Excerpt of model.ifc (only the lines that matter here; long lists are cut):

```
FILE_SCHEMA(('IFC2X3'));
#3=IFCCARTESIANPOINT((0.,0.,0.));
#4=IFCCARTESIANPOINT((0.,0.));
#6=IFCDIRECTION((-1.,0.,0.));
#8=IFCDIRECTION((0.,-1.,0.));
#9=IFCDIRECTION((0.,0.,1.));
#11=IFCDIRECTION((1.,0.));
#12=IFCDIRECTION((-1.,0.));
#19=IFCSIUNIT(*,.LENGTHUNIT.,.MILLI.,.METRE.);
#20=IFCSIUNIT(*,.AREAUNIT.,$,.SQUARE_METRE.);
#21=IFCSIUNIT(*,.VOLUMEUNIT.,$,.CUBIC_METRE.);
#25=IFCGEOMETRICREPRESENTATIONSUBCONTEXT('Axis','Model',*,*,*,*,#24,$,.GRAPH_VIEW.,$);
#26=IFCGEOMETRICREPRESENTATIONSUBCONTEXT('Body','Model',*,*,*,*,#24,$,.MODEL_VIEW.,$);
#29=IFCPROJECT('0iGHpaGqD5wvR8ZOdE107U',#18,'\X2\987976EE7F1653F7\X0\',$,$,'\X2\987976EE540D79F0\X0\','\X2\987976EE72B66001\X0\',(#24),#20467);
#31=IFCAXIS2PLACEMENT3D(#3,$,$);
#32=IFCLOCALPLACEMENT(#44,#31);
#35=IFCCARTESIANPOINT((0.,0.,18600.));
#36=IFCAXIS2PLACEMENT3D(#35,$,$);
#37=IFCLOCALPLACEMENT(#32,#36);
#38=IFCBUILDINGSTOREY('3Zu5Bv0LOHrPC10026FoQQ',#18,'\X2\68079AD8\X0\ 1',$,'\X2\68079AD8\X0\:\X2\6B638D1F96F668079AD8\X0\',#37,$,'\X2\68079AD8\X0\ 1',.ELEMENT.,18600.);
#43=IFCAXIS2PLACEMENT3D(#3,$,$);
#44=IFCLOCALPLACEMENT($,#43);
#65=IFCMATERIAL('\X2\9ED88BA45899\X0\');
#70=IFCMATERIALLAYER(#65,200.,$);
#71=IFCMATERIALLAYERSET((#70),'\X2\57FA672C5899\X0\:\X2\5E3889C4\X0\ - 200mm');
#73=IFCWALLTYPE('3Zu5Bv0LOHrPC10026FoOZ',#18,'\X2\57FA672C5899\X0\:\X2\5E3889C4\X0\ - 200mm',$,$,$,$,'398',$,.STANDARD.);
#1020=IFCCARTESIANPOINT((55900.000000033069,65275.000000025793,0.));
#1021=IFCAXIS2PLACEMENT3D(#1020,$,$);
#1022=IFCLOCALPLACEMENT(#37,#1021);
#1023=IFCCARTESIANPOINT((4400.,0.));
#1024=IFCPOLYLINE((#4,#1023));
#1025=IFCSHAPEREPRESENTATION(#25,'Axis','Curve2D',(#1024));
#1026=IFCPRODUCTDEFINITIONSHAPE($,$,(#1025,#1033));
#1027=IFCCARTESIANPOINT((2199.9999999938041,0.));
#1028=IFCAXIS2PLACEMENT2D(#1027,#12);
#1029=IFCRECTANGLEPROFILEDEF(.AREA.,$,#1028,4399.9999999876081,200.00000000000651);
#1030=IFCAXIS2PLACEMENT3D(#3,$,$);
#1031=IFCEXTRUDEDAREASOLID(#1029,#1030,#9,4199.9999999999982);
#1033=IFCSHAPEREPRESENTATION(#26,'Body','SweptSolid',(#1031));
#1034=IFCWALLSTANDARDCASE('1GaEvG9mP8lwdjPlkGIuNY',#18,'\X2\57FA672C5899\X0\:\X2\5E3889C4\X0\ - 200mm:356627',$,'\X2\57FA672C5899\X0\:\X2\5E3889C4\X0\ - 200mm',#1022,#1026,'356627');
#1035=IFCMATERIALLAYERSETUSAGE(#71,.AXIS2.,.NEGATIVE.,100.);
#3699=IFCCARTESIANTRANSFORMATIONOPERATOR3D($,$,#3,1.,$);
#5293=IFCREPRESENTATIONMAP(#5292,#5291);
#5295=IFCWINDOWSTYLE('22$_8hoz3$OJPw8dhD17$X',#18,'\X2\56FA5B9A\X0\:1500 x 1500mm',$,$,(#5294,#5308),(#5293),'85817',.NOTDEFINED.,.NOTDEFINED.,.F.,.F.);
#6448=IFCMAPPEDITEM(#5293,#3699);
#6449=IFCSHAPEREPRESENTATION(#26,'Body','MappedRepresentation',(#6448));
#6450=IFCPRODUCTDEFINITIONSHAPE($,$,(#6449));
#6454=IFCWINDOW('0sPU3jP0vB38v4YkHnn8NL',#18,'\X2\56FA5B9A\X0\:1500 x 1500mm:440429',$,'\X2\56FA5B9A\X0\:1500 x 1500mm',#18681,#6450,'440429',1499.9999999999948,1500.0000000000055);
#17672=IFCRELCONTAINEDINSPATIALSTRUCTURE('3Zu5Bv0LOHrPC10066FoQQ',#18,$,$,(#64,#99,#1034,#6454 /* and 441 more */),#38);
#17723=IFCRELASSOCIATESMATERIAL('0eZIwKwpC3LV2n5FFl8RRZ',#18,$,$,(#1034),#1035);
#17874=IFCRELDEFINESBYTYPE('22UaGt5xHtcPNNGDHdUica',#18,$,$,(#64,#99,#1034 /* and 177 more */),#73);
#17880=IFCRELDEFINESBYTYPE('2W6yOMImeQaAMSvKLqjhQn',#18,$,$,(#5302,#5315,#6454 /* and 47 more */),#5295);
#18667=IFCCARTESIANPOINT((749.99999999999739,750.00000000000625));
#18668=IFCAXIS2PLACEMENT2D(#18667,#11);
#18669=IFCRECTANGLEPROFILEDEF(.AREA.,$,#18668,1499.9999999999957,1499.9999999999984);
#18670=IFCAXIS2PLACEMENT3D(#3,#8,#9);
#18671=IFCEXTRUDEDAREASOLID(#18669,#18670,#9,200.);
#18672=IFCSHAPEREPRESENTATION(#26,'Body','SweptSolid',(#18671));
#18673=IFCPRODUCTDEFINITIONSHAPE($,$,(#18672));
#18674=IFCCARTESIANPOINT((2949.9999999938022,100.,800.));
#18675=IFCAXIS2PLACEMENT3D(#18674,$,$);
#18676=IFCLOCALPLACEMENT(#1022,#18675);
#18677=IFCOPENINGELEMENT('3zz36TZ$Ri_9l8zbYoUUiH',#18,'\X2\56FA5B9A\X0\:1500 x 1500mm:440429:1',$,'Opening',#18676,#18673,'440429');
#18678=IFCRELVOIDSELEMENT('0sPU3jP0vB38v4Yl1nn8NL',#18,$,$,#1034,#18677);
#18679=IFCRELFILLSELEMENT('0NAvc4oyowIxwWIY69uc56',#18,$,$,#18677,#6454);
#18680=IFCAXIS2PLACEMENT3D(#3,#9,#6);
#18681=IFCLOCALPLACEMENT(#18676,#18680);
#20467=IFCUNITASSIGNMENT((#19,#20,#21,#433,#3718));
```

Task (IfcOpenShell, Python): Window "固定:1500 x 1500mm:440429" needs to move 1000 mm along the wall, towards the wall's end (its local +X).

```python
import ifcopenshell
import ifcopenshell.api.geometry
import ifcopenshell.util.placement
import ifcopenshell.util.unit

model = ifcopenshell.open("model.ifc")
unit_scale = ifcopenshell.util.unit.calculate_unit_scale(model)

window = model.by_id(6454)
opening = window.FillsVoids[0].RelatingOpeningElement
wall = opening.VoidsElements[0].RelatingBuildingElement

wall_matrix = ifcopenshell.util.placement.get_local_placement(wall.ObjectPlacement)
shift = wall_matrix[:3, 0] * 1 / unit_scale
before = ifcopenshell.util.placement.get_local_placement(window.ObjectPlacement)[:3, 3].copy()

# The window is placed relative to its opening, so it follows when the opening moves.
matrix = ifcopenshell.util.placement.get_local_placement(opening.ObjectPlacement)
matrix[:3, 3] += shift
ifcopenshell.api.geometry.edit_object_placement(
    model, product=opening, matrix=matrix, is_si=False, should_transform_children=True
)

after = ifcopenshell.util.placement.get_local_placement(window.ObjectPlacement)[:3, 3]
print("window moved by", (after - before).round(3) + 0.0)

model.write("model-out.ifc")
```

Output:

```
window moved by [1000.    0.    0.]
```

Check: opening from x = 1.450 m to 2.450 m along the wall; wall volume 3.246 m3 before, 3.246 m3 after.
